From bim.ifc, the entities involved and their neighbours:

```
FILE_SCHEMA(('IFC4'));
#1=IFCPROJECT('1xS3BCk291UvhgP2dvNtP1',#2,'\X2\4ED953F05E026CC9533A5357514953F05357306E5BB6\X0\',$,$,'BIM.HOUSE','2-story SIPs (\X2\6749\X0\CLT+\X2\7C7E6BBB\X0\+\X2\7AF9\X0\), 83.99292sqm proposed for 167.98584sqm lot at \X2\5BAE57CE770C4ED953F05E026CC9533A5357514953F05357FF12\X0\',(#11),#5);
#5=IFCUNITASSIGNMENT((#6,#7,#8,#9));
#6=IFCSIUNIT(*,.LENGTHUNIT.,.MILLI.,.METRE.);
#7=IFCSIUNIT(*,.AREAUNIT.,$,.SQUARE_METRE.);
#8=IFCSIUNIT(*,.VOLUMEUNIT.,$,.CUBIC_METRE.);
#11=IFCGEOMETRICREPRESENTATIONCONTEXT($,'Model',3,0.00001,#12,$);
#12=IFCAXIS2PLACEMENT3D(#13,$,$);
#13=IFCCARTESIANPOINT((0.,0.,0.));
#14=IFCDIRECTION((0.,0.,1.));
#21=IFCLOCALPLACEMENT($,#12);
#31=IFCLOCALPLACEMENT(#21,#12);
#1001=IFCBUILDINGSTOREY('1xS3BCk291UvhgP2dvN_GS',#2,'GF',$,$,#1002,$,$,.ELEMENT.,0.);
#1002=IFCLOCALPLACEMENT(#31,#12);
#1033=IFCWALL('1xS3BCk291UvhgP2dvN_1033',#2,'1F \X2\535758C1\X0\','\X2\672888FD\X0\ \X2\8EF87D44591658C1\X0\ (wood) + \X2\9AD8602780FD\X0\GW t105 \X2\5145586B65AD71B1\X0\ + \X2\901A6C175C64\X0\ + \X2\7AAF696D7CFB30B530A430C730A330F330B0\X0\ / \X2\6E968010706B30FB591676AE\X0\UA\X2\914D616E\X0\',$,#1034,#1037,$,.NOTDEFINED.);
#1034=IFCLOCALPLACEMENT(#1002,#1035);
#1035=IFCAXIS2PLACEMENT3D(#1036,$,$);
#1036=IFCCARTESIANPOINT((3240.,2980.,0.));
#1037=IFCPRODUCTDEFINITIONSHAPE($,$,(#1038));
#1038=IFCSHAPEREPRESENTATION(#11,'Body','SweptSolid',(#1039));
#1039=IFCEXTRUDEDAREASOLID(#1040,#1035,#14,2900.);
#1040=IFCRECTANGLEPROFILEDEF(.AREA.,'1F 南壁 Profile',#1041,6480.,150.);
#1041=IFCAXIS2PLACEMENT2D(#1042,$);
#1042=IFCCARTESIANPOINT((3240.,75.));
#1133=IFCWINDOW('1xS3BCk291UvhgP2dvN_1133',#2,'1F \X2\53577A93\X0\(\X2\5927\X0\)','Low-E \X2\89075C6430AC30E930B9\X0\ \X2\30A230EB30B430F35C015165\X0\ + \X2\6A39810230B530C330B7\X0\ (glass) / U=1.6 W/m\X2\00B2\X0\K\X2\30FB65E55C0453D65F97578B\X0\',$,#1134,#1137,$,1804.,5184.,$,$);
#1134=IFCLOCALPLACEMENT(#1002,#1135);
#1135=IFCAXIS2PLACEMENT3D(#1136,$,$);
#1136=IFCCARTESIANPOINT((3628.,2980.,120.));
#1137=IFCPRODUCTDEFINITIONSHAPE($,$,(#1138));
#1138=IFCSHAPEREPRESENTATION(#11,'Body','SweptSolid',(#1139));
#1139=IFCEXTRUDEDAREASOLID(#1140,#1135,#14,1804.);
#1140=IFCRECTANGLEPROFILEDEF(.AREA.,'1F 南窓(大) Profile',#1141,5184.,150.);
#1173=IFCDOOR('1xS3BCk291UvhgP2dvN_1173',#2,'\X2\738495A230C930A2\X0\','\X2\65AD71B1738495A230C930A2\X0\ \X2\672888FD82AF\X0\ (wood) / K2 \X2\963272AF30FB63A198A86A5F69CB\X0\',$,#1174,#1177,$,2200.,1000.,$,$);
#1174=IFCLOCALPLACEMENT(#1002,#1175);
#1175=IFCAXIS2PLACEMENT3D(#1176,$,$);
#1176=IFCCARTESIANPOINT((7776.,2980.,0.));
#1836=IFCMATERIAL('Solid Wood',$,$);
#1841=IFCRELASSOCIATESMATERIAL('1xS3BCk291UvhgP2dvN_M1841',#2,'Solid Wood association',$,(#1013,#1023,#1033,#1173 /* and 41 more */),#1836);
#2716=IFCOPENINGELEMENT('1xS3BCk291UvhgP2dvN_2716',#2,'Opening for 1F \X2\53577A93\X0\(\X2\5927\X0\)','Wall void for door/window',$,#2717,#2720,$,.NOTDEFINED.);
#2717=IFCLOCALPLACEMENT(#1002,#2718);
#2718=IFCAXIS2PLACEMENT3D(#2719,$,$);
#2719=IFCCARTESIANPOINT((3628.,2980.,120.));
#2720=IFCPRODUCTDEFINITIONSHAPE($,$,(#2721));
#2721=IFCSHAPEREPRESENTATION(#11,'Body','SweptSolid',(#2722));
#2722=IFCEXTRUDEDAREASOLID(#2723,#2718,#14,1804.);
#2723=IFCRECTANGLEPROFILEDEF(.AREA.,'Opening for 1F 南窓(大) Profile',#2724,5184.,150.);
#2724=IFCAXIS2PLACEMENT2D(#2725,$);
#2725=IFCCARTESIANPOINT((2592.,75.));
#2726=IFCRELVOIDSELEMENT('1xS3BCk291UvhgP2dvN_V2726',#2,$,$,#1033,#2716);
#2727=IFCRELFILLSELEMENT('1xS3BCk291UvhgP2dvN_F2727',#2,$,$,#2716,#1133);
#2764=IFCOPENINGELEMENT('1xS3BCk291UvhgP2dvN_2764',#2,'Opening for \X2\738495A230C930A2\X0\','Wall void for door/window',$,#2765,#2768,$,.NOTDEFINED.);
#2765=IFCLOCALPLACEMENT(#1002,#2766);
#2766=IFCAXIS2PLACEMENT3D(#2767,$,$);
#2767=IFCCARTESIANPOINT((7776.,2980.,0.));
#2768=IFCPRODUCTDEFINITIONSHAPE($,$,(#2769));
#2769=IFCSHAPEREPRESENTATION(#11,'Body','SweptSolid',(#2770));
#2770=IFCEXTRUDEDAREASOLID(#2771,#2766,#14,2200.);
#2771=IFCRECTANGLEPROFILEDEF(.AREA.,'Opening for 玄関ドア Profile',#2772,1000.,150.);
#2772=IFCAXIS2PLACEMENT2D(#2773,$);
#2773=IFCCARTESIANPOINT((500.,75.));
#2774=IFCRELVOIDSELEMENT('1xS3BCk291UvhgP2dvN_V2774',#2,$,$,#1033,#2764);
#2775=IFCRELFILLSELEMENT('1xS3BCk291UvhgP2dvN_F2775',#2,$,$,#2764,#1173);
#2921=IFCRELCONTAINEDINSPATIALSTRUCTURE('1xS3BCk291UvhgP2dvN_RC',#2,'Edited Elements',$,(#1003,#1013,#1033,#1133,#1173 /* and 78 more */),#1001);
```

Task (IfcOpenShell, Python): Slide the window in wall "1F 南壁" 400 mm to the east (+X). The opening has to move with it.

```python
import ifcopenshell
import ifcopenshell.api.geometry
import ifcopenshell.util.placement
import ifcopenshell.util.unit

model = ifcopenshell.open("bim.ifc")
unit_scale = ifcopenshell.util.unit.calculate_unit_scale(model)

window = model.by_id(1133)
opening = window.FillsVoids[0].RelatingOpeningElement
wall = opening.VoidsElements[0].RelatingBuildingElement

wall_matrix = ifcopenshell.util.placement.get_local_placement(wall.ObjectPlacement)
shift = wall_matrix[:3, 0] * 0.4 / unit_scale
before = ifcopenshell.util.placement.get_local_placement(window.ObjectPlacement)[:3, 3].copy()

# The window is not placed relative to its opening, so move both.
for product in (opening, window):
    matrix = ifcopenshell.util.placement.get_local_placement(product.ObjectPlacement)
    matrix[:3, 3] += shift
    ifcopenshell.api.geometry.edit_object_placement(model, product=product, matrix=matrix, is_si=False)

after = ifcopenshell.util.placement.get_local_placement(window.ObjectPlacement)[:3, 3]
print("window moved by", (after - before).round(3) + 0.0)

model.write("bim_updated.ifc")
```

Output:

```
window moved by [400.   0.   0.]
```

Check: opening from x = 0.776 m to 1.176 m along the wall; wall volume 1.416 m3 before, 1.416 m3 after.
